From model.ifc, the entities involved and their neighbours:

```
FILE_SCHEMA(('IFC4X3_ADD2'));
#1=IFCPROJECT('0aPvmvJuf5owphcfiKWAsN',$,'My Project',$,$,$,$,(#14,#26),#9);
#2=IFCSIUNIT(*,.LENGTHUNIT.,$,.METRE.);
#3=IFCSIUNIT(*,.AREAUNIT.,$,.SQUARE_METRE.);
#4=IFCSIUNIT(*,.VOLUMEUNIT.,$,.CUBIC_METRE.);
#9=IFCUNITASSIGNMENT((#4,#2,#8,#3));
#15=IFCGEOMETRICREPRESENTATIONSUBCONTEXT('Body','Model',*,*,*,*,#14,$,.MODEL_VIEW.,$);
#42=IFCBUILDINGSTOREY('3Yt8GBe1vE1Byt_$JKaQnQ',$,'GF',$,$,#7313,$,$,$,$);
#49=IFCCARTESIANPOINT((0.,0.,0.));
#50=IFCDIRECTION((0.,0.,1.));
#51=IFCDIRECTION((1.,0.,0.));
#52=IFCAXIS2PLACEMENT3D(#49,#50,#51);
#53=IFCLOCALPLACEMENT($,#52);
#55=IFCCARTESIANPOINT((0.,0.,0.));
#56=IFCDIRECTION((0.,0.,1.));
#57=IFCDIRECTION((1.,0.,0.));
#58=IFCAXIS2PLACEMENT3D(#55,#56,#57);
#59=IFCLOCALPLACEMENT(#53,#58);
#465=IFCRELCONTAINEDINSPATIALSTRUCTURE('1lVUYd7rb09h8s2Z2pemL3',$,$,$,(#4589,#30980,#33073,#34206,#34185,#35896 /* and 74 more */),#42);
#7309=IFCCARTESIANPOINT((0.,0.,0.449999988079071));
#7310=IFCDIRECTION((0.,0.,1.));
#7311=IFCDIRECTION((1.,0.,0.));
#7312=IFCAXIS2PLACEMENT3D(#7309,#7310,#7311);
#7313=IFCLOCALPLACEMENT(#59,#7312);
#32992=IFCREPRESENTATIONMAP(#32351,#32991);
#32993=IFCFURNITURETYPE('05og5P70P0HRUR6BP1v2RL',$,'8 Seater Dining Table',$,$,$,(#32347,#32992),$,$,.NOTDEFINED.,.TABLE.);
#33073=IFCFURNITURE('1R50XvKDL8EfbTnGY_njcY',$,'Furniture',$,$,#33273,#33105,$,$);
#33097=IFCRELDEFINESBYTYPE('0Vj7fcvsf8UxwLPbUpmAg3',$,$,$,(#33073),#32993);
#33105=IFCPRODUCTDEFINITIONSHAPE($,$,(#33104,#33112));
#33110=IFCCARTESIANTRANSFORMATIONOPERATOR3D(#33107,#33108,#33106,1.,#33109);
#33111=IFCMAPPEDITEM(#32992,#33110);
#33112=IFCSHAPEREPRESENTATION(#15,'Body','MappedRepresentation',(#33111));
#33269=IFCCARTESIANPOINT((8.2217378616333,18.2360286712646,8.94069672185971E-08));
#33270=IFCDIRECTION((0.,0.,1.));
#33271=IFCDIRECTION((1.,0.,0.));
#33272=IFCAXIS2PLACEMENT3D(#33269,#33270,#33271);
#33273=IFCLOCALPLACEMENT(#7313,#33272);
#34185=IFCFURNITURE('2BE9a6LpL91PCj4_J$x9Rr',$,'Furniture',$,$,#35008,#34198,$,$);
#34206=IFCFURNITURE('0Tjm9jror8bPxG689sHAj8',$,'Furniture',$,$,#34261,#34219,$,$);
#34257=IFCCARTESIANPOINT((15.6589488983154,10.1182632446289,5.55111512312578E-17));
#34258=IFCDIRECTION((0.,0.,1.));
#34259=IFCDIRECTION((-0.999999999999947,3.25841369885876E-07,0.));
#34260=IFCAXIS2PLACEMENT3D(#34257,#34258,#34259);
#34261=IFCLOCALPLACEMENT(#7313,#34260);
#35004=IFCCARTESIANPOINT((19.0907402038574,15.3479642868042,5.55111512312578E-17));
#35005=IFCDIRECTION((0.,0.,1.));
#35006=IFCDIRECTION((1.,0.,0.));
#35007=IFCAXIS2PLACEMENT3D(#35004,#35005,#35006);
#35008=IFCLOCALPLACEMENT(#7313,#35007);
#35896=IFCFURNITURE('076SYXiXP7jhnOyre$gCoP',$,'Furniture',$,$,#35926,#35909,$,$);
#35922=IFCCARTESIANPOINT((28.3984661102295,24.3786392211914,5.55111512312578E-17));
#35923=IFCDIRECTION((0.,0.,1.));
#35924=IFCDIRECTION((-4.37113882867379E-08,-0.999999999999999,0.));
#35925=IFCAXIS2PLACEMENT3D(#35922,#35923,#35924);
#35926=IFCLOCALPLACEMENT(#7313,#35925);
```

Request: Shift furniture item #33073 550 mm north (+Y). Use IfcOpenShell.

```python
import ifcopenshell
import ifcopenshell.api.geometry
import ifcopenshell.util.placement
import ifcopenshell.util.unit

model = ifcopenshell.open("model.ifc")
unit_scale = ifcopenshell.util.unit.calculate_unit_scale(model)

item = model.by_guid("1R50XvKDL8EfbTnGY_njcY")
matrix = ifcopenshell.util.placement.get_local_placement(item.ObjectPlacement)
matrix[1, 3] += 0.55 / unit_scale
ifcopenshell.api.geometry.edit_object_placement(model, product=item, matrix=matrix, is_si=False)

print(ifcopenshell.util.placement.get_local_placement(item.ObjectPlacement).round(3) + 0.0)

model.write("model-out.ifc")
```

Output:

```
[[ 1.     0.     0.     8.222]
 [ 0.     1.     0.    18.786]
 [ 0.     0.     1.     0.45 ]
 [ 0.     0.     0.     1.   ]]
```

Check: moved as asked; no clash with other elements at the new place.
